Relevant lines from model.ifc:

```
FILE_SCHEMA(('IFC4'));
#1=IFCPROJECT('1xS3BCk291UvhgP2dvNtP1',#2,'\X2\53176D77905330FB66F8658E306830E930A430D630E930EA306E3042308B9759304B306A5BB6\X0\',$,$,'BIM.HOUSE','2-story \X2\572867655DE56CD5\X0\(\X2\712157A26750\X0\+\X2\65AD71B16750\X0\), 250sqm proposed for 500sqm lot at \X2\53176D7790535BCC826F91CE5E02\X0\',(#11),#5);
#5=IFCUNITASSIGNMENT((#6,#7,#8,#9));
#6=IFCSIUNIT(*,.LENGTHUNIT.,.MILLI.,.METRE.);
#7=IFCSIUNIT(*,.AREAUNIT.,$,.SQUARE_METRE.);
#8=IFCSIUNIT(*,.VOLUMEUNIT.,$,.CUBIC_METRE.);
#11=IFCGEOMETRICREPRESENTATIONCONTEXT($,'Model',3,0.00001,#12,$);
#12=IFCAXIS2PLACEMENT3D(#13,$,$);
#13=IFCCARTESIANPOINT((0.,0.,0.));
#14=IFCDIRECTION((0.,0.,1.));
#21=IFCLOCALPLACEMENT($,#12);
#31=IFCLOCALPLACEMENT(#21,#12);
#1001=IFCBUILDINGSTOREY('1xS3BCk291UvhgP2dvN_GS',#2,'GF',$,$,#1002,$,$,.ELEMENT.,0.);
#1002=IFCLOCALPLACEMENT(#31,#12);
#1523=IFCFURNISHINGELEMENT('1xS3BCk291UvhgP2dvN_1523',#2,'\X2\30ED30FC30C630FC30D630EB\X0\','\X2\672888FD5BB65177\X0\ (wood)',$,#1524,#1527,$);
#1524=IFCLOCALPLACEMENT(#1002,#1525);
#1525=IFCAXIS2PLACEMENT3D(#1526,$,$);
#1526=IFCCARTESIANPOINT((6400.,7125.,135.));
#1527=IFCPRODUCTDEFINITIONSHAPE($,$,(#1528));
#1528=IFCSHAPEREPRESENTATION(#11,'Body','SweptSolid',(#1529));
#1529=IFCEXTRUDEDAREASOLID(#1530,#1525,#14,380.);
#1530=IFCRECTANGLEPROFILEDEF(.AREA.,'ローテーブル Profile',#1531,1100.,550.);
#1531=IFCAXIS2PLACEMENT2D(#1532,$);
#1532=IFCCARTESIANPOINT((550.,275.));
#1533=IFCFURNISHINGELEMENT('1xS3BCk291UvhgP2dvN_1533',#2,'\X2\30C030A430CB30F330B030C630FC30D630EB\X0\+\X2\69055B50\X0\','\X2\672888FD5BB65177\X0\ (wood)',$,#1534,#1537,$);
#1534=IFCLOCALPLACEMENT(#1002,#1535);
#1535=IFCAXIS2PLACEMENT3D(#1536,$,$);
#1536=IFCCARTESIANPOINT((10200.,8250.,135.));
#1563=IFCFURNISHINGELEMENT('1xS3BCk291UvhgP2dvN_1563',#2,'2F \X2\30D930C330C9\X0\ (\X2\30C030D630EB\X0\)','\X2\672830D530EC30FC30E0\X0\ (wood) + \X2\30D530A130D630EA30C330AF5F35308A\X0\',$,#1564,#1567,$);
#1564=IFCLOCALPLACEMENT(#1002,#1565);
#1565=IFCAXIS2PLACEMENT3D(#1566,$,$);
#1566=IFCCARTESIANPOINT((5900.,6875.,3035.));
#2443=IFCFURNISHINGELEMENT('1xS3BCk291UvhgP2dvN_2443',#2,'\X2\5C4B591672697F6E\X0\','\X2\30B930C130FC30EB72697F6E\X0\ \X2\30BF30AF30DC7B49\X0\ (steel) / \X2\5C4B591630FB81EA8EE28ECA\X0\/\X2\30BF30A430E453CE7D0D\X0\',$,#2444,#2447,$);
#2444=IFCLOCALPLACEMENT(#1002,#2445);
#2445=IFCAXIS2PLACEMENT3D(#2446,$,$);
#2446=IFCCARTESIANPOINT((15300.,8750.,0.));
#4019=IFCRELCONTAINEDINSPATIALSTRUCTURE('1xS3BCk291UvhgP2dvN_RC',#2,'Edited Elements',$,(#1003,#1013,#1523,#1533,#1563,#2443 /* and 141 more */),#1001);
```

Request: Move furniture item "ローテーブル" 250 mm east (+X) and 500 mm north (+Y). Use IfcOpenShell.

```python
import ifcopenshell
import ifcopenshell.api.geometry
import ifcopenshell.util.placement
import ifcopenshell.util.unit

model = ifcopenshell.open("model.ifc")
unit_scale = ifcopenshell.util.unit.calculate_unit_scale(model)

item = model.by_id(1523)
matrix = ifcopenshell.util.placement.get_local_placement(item.ObjectPlacement)
matrix[0, 3] += 0.25 / unit_scale
matrix[1, 3] += 0.5 / unit_scale
ifcopenshell.api.geometry.edit_object_placement(model, product=item, matrix=matrix, is_si=False)

print(ifcopenshell.util.placement.get_local_placement(item.ObjectPlacement).round(3) + 0.0)

model.write("model_edited.ifc")
```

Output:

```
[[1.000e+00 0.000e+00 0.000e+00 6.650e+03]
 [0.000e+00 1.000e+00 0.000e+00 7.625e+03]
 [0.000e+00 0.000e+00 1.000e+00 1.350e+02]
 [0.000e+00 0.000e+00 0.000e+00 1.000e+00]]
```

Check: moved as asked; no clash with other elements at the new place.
